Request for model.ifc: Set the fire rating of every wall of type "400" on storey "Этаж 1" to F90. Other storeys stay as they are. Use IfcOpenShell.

First a look at what the model holds.

```python
import ifcopenshell
import ifcopenshell.util.element

model = ifcopenshell.open("model.ifc")
print(model.schema)
storey = next(s for s in model.by_type("IfcBuildingStorey") if s.Name == "Этаж 1")
walls = [e for e in ifcopenshell.util.element.get_decomposition(storey) if e.is_a("IfcWall")]
seen = {}
for e in walls:
    element_type = ifcopenshell.util.element.get_type(e)
    key = (element_type.Name if element_type != e and element_type else None, ifcopenshell.util.element.get_pset(e, "Pset_WallCommon", "FireRating"))
    seen[key] = seen.get(key, 0) + 1
for (name, value), count in sorted(seen.items(), key=str):
    print(count, "x", name, "|", value)
```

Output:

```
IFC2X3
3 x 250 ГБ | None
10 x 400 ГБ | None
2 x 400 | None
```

```python
import ifcopenshell
import ifcopenshell.api.pset
import ifcopenshell.util.element

model = ifcopenshell.open("model.ifc")

storey = next(s for s in model.by_type("IfcBuildingStorey") if s.Name == "Этаж 1")
walls = [e for e in ifcopenshell.util.element.get_decomposition(storey) if e.is_a("IfcWall")]

count = 0
for e in walls:
    element_type = ifcopenshell.util.element.get_type(e)
    if element_type in (None, e) or element_type.Name != "400":
        continue
    # add_pset returns the element's existing set when there is one.
    pset = ifcopenshell.api.pset.add_pset(model, product=e, name="Pset_WallCommon")
    ifcopenshell.api.pset.edit_pset(model, pset=pset, properties={"FireRating": "F90"})
    count += 1

print(count, "walls updated")

model.write("model_edited.ifc")
```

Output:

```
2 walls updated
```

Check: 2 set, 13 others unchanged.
